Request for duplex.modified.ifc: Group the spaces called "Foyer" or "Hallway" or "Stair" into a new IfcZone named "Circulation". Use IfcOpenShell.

First a look at what the model holds.

```python
import ifcopenshell

model = ifcopenshell.open("duplex.modified.ifc")
print(model.schema)
seen = {}
for space in model.by_type("IfcSpace"):
    seen[space.LongName] = seen.get(space.LongName, 0) + 1
for name, count in sorted(seen.items(), key=str):
    print(count, "x", name)
print("zones:", [z.Name for z in model.by_type("IfcZone")][:20])
```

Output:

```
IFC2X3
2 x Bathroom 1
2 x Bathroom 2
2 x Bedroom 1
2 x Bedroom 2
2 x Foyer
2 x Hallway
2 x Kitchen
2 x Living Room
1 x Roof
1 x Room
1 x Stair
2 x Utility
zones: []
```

```python
import ifcopenshell
import ifcopenshell.api.group
import ifcopenshell.api.root

model = ifcopenshell.open("duplex.modified.ifc")

names = {"Foyer", "Hallway", "Stair"}
spaces = [s for s in model.by_type("IfcSpace") if s.LongName in names]

zone = ifcopenshell.api.root.create_entity(model, ifc_class="IfcZone", name="Circulation")
ifcopenshell.api.group.assign_group(model, products=spaces, group=zone)
print(len(spaces), "spaces in", zone.Name)

model.write("duplex.modified-out.ifc")
```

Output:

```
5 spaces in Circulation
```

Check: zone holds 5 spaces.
